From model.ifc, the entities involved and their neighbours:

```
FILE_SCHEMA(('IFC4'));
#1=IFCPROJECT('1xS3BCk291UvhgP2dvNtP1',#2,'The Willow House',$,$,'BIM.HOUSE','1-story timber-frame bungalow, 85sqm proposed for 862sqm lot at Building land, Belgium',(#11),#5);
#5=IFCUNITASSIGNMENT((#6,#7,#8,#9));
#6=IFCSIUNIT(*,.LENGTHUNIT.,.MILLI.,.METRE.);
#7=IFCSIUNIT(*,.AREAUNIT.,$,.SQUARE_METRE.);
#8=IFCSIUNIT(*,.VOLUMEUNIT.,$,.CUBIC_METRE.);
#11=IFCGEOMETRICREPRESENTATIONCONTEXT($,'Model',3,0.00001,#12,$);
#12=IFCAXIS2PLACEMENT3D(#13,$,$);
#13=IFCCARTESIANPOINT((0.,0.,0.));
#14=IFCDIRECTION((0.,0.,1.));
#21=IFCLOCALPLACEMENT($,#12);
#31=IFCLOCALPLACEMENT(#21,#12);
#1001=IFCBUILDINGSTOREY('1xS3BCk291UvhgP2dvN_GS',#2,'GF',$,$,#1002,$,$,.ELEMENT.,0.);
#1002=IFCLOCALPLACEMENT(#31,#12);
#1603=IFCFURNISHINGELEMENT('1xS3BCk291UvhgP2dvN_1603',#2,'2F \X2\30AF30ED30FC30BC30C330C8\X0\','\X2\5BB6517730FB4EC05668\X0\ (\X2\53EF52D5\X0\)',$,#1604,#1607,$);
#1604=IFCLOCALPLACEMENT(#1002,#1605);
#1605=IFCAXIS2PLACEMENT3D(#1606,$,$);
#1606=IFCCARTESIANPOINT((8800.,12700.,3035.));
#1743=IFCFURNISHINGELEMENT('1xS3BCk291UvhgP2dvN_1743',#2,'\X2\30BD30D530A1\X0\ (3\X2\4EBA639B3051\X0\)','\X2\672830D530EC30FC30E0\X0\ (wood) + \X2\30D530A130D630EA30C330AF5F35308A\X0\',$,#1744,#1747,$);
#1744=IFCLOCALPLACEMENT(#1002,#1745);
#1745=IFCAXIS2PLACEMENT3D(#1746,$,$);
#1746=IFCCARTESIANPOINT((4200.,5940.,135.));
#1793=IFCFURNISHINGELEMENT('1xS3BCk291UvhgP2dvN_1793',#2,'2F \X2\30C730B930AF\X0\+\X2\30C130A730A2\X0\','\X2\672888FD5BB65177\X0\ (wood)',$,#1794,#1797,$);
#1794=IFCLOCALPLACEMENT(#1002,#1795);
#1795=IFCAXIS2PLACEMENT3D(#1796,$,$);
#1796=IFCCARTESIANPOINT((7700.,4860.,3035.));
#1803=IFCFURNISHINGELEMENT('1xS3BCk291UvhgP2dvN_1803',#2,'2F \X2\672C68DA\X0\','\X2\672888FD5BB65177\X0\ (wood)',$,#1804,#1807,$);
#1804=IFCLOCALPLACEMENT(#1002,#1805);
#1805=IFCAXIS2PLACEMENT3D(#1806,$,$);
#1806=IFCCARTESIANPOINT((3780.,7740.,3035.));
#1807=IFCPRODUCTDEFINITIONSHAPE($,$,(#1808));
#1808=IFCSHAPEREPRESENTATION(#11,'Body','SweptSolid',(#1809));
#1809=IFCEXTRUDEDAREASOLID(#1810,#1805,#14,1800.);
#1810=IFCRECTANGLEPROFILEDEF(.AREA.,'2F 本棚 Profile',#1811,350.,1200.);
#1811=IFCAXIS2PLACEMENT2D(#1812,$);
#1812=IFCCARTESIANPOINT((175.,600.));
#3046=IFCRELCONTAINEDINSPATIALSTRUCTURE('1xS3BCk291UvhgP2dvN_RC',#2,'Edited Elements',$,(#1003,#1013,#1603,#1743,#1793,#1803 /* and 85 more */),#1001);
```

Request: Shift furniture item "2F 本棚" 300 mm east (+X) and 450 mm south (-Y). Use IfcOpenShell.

```python
import ifcopenshell
import ifcopenshell.api.geometry
import ifcopenshell.util.placement
import ifcopenshell.util.unit

model = ifcopenshell.open("model.ifc")
unit_scale = ifcopenshell.util.unit.calculate_unit_scale(model)

item = model.by_guid("1xS3BCk291UvhgP2dvN_1803")
matrix = ifcopenshell.util.placement.get_local_placement(item.ObjectPlacement)
matrix[0, 3] += 0.3 / unit_scale
matrix[1, 3] -= 0.45 / unit_scale
ifcopenshell.api.geometry.edit_object_placement(model, product=item, matrix=matrix, is_si=False)

print(ifcopenshell.util.placement.get_local_placement(item.ObjectPlacement).round(3) + 0.0)

model.write("model-out.ifc")
```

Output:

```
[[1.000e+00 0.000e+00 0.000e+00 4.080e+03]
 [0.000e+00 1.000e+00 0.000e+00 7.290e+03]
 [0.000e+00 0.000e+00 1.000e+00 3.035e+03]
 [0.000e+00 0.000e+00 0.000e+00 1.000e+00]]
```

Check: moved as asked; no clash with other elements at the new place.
